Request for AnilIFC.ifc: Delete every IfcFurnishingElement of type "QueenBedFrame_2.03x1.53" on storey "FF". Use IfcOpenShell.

First a look at what the model holds.

```python
import ifcopenshell
import ifcopenshell.util.element

model = ifcopenshell.open("AnilIFC.ifc")
print(model.schema)
storey = next(s for s in model.by_type("IfcBuildingStorey") if s.Name == "FF")
furniture = [e for e in ifcopenshell.util.element.get_decomposition(storey) if e.is_a("IfcFurnishingElement")]
seen = {}
for e in furniture:
    element_type = ifcopenshell.util.element.get_type(e)
    name = element_type.Name if element_type not in (None, e) else None
    seen[name] = seen.get(name, 0) + 1
for name, count in sorted(seen.items(), key=str):
    print(count, "x", name)
```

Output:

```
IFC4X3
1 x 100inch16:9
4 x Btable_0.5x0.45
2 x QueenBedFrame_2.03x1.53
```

```python
import ifcopenshell
import ifcopenshell.api.root
import ifcopenshell.util.element

model = ifcopenshell.open("AnilIFC.ifc")

storey = next(s for s in model.by_type("IfcBuildingStorey") if s.Name == "FF")
furniture = [e for e in ifcopenshell.util.element.get_decomposition(storey) if e.is_a("IfcFurnishingElement")]
targets = [e for e in furniture if (t := ifcopenshell.util.element.get_type(e)) not in (None, e) and t.Name == "QueenBedFrame_2.03x1.53"]

for e in targets:
    ifcopenshell.api.root.remove_product(model, product=e)
print(len(targets), "removed")

model.write("AnilIFC_v2.ifc")
```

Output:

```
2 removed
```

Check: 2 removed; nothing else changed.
